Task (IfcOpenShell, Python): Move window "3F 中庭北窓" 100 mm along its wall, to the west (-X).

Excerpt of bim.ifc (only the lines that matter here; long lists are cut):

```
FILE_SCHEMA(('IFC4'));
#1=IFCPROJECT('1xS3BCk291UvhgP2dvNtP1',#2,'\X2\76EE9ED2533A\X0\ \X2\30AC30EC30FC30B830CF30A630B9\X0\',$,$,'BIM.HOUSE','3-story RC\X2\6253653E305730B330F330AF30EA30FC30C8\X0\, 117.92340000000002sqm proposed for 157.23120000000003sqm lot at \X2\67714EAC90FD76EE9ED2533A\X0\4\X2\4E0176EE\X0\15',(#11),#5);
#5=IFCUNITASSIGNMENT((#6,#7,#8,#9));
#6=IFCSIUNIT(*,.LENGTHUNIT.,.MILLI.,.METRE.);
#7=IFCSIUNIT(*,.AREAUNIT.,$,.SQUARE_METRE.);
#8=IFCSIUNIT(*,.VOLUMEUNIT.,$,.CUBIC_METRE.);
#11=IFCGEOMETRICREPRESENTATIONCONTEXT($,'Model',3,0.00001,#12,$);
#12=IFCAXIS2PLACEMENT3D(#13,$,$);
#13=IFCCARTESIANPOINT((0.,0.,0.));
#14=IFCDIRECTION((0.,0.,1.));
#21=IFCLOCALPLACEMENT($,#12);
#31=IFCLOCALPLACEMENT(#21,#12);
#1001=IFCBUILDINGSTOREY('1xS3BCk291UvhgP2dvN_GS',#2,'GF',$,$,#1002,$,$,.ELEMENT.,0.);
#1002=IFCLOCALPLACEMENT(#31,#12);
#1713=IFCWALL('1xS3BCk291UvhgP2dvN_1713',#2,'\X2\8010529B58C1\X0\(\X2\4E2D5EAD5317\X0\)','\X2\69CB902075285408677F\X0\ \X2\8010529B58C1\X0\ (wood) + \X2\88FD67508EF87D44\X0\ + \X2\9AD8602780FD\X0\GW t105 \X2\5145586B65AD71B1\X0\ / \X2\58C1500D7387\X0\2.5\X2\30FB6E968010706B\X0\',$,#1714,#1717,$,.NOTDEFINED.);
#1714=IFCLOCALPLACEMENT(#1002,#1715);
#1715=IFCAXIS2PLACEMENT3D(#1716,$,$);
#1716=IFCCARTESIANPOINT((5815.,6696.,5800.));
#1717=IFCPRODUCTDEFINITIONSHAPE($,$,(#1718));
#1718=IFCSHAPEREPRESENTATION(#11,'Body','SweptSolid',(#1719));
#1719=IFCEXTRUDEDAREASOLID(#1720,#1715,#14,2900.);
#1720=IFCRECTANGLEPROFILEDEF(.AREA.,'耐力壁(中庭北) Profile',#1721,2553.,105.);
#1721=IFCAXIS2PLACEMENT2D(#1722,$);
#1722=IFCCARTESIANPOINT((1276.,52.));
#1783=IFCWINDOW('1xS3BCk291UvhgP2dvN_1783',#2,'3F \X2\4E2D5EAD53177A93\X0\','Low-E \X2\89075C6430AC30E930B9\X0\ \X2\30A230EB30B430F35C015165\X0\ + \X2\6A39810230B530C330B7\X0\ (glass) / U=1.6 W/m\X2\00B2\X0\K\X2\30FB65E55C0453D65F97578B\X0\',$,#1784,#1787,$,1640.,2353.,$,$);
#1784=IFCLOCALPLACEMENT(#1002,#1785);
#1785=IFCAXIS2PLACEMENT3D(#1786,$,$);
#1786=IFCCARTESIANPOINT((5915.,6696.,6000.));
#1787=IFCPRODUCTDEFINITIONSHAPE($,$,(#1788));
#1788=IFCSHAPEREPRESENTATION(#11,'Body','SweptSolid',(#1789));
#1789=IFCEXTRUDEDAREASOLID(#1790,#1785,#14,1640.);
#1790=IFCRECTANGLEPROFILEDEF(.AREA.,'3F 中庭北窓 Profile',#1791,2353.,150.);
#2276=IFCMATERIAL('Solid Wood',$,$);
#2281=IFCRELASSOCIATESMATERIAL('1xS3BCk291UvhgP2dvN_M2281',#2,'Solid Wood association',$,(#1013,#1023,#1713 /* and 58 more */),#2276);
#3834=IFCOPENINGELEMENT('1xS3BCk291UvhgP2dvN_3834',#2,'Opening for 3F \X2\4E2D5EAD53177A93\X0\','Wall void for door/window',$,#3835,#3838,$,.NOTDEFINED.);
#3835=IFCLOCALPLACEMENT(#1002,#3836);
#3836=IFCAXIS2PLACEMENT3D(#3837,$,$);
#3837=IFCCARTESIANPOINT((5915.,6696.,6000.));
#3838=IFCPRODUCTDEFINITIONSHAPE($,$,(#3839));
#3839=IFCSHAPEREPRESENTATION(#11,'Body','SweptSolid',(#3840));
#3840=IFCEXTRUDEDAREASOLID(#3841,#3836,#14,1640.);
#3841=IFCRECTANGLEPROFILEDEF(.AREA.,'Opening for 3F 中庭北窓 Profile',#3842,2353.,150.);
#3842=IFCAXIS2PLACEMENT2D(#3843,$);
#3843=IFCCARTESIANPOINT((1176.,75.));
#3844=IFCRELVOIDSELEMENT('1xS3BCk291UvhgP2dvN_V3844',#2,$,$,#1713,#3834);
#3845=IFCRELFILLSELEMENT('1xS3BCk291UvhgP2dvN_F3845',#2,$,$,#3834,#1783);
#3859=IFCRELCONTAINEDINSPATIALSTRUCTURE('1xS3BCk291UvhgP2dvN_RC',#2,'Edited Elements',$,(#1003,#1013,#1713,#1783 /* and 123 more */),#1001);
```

```python
import ifcopenshell
import ifcopenshell.api.geometry
import ifcopenshell.util.placement

model = ifcopenshell.open("bim.ifc")

window = model.by_guid("1xS3BCk291UvhgP2dvN_1783")
opening = window.FillsVoids[0].RelatingOpeningElement
wall = opening.VoidsElements[0].RelatingBuildingElement

wall_matrix = ifcopenshell.util.placement.get_local_placement(wall.ObjectPlacement)
shift = wall_matrix[:3, 0] * -100.0
before = ifcopenshell.util.placement.get_local_placement(window.ObjectPlacement)[:3, 3].copy()

# The window is not placed relative to its opening, so move both.
for product in (opening, window):
    matrix = ifcopenshell.util.placement.get_local_placement(product.ObjectPlacement)
    matrix[:3, 3] += shift
    ifcopenshell.api.geometry.edit_object_placement(model, product=product, matrix=matrix, is_si=False)

after = ifcopenshell.util.placement.get_local_placement(window.ObjectPlacement)[:3, 3]
print("window moved by", (after - before).round(3) + 0.0)

model.write("bim_rev.ifc")
```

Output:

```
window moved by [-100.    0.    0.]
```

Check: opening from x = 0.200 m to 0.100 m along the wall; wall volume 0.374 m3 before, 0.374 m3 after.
